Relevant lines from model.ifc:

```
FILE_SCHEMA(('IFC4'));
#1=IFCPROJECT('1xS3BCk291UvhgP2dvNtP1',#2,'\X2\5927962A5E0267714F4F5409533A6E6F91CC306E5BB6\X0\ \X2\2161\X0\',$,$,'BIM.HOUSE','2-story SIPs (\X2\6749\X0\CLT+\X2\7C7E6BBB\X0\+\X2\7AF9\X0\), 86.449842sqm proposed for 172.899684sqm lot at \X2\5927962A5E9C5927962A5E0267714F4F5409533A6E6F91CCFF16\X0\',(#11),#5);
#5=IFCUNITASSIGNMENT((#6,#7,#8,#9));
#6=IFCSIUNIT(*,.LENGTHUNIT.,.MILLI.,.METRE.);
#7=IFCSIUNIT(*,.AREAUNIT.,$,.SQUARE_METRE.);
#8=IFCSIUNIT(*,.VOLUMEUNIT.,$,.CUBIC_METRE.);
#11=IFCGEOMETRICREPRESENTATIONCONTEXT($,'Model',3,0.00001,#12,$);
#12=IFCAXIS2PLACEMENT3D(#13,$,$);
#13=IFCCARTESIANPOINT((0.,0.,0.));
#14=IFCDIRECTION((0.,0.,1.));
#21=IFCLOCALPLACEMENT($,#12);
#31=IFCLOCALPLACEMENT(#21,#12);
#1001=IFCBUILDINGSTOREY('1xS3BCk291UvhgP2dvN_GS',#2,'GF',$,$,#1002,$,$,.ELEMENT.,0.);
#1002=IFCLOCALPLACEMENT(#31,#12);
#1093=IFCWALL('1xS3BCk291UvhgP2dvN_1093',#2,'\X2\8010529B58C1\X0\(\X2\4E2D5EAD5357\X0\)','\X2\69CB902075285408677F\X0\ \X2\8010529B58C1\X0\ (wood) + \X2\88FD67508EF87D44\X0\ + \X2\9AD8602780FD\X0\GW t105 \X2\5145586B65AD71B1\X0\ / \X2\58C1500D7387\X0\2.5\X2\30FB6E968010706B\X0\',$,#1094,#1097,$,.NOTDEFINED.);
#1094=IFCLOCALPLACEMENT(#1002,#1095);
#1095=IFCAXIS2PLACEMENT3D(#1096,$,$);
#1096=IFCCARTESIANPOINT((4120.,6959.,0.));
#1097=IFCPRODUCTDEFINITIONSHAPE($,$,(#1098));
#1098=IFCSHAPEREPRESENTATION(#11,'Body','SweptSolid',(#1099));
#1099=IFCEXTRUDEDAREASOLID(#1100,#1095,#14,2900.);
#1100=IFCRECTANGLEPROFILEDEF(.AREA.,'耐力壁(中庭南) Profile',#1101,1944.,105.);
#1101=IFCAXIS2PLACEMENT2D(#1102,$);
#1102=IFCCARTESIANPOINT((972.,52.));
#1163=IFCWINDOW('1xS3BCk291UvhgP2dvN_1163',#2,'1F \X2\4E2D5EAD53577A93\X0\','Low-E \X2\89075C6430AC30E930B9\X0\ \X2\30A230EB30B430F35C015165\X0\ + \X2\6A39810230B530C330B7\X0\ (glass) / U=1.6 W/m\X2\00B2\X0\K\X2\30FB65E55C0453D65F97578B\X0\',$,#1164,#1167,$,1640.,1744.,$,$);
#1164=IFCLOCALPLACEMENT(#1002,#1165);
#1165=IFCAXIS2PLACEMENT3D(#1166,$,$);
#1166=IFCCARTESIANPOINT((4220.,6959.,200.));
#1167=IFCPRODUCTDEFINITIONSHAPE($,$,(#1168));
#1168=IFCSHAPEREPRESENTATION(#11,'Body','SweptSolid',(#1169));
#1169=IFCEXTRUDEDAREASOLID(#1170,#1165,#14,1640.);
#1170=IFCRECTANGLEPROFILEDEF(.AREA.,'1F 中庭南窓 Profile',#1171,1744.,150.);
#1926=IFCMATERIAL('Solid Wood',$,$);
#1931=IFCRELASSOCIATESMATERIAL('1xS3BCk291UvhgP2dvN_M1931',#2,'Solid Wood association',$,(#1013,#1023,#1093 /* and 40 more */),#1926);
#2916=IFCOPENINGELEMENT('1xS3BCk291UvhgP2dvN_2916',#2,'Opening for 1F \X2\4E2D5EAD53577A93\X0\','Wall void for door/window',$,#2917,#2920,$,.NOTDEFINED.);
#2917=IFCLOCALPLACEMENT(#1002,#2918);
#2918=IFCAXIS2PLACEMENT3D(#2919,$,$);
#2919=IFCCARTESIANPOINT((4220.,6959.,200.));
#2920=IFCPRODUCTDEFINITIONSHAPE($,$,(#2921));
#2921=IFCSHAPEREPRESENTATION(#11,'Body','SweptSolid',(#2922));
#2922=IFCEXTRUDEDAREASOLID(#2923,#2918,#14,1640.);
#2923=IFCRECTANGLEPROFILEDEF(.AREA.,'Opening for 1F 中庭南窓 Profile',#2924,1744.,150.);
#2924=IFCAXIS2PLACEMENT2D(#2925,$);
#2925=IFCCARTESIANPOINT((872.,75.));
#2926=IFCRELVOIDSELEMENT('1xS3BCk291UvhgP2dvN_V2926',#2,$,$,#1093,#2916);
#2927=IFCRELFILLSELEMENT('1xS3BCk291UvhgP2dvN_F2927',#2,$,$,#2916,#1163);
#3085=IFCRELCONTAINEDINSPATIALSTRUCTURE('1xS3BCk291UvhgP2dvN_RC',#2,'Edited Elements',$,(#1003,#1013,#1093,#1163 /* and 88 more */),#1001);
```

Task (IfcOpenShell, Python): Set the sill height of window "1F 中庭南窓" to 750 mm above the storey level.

```python
import numpy as np
import ifcopenshell
import ifcopenshell.api.geometry
import ifcopenshell.geom
import ifcopenshell.util.element
import ifcopenshell.util.placement
import ifcopenshell.util.shape
import ifcopenshell.util.unit

model = ifcopenshell.open("model.ifc")
unit_scale = ifcopenshell.util.unit.calculate_unit_scale(model)

window = model.by_guid("1xS3BCk291UvhgP2dvN_1163")
opening = window.FillsVoids[0].RelatingOpeningElement
storey = ifcopenshell.util.element.get_container(window, ifc_class="IfcBuildingStorey")
level = ifcopenshell.util.placement.get_local_placement(storey.ObjectPlacement)[2, 3]

# The opening's origin need not be at the sill, so measure its lowest point.
shape = ifcopenshell.geom.create_shape(ifcopenshell.geom.settings(), opening)
bottom = ifcopenshell.util.shape.get_shape_bottom_elevation(shape, shape.geometry) / unit_scale
dz = level + 750.0 - bottom

shift = np.array([0.0, 0.0, dz])
# The window is not placed relative to its opening, so move both.
for product in (opening, window):
    matrix = ifcopenshell.util.placement.get_local_placement(product.ObjectPlacement)
    matrix[:3, 3] += shift
    ifcopenshell.api.geometry.edit_object_placement(model, product=product, matrix=matrix, is_si=False)

print(f"moved by {dz * unit_scale:+.3f} m")

model.write("model_updated.ifc")
```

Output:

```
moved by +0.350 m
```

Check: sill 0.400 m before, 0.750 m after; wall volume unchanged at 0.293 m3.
